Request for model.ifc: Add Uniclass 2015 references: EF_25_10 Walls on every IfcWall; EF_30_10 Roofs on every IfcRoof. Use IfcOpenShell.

First a look at what the model holds.

```python
import ifcopenshell

model = ifcopenshell.open("model.ifc")
print(model.schema)
print("classifications:", [c.Name for c in model.by_type("IfcClassification")])
for ifc_class in ("IfcDoor", "IfcRoof", "IfcStair", "IfcWall", "IfcWindow"):
    print(ifc_class, len(model.by_type(ifc_class)))
```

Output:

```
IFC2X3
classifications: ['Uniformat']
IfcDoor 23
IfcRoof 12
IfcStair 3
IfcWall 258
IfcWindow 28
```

```python
import ifcopenshell
import ifcopenshell.api.classification

model = ifcopenshell.open("model.ifc")

# IFC2X3 requires Source and Edition and has no link from the project to the system.
system = model.create_entity("IfcClassification", Source="NBS", Edition="2015", Name="Uniclass 2015")

codes = {
    "IfcWall": ("EF_25_10", "Walls"),
    "IfcRoof": ("EF_30_10", "Roofs"),
}
for ifc_class, (code, name) in codes.items():
    products = model.by_type(ifc_class)
    ifcopenshell.api.classification.add_reference(
        model, products=products, classification=system, identification=code, name=name
    )
    print(code, len(products))

model.write("model_rev.ifc")
```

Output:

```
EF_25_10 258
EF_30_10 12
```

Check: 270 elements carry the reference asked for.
